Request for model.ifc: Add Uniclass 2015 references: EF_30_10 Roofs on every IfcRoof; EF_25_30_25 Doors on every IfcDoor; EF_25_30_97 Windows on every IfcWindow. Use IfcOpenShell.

First a look at what the model holds.

```python
import ifcopenshell

model = ifcopenshell.open("model.ifc")
print(model.schema)
print("classifications:", [c.Name for c in model.by_type("IfcClassification")])
for ifc_class in ("IfcDoor", "IfcRoof", "IfcStair", "IfcWall", "IfcWindow"):
    print(ifc_class, len(model.by_type(ifc_class)))
```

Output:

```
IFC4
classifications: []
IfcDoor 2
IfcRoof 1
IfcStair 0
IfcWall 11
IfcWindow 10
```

```python
import ifcopenshell
import ifcopenshell.api.classification

model = ifcopenshell.open("model.ifc")

system = ifcopenshell.api.classification.add_classification(model, classification="Uniclass 2015")

codes = {
    "IfcRoof": ("EF_30_10", "Roofs"),
    "IfcDoor": ("EF_25_30_25", "Doors"),
    "IfcWindow": ("EF_25_30_97", "Windows"),
}
for ifc_class, (code, name) in codes.items():
    products = model.by_type(ifc_class)
    ifcopenshell.api.classification.add_reference(
        model, products=products, classification=system, identification=code, name=name
    )
    print(code, len(products))

model.write("model_rev.ifc")
```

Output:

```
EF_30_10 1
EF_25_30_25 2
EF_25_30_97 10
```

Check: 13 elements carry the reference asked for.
